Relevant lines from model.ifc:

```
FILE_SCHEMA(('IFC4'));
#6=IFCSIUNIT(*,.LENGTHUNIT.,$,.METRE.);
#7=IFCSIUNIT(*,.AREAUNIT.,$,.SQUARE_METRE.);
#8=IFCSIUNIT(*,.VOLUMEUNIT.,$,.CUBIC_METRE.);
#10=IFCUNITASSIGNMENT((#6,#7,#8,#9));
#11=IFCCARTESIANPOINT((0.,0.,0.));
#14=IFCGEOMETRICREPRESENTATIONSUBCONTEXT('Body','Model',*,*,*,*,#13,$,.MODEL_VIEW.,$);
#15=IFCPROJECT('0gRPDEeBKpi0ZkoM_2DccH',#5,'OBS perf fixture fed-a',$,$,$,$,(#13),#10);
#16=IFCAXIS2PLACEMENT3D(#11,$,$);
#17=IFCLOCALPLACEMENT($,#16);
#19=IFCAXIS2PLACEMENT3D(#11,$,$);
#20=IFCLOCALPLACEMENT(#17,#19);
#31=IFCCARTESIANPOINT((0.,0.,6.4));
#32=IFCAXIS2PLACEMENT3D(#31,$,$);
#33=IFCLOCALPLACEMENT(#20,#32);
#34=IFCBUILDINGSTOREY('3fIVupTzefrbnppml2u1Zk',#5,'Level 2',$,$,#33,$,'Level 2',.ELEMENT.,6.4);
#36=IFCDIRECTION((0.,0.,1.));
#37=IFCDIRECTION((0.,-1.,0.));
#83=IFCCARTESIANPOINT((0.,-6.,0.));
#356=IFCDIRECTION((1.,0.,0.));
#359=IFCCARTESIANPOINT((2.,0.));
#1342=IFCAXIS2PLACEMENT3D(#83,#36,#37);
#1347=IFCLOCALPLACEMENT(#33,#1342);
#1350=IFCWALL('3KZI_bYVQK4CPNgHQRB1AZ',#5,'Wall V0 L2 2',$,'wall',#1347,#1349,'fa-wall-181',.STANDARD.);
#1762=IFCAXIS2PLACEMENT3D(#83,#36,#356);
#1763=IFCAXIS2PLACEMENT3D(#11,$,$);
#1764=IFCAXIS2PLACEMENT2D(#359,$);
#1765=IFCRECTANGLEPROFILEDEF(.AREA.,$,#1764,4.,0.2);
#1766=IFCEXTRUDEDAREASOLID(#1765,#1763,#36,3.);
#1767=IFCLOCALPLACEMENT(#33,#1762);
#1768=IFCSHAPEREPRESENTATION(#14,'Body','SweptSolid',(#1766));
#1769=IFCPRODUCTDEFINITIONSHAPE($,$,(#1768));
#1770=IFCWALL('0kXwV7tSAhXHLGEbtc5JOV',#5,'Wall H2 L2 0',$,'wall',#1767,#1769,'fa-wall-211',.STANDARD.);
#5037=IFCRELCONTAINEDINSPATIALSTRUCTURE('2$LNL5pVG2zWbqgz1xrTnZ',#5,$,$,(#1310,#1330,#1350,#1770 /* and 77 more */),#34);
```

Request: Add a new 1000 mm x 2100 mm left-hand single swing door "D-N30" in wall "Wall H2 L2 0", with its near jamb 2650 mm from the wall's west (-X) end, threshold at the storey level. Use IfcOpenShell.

```python
import numpy as np
import ifcopenshell
import ifcopenshell.api.feature
import ifcopenshell.api.geometry
import ifcopenshell.api.root
import ifcopenshell.api.spatial
import ifcopenshell.geom
import ifcopenshell.util.element
import ifcopenshell.util.placement
import ifcopenshell.util.representation
import ifcopenshell.util.shape
import ifcopenshell.util.unit

model = ifcopenshell.open("model.ifc")
unit_scale = ifcopenshell.util.unit.calculate_unit_scale(model)
settings = ifcopenshell.geom.settings()


def volume(element):
    """Net volume in cubic metres, openings subtracted."""
    shape = ifcopenshell.geom.create_shape(settings, element)
    return ifcopenshell.util.shape.get_volume(shape.geometry)


wall = model.by_guid("0kXwV7tSAhXHLGEbtc5JOV")
storey = ifcopenshell.util.element.get_container(wall, ifc_class="IfcBuildingStorey")
context = ifcopenshell.util.representation.get_context(model, "Model", "Body", "MODEL_VIEW")
before = volume(wall)

width, height, from_end, sill = 1, 2.1, 2.65, 0.0  # metres

# The wall runs along its own X axis, and the end named is its -X end.
wall_shape = ifcopenshell.geom.create_shape(settings, wall)
x, y, z = ifcopenshell.util.shape.get_vertices(wall_shape.geometry).T
start = x.min() + from_end
face, thickness = float(y.min()), float(y.max() - y.min())
wall_matrix = ifcopenshell.util.placement.get_local_placement(wall.ObjectPlacement)
level = ifcopenshell.util.placement.get_local_placement(storey.ObjectPlacement)[2, 3]


def in_wall(x, y):
    """Placement at x, y metres in the wall's axes, at sill height."""
    matrix = wall_matrix.copy()
    matrix[:, 3] = wall_matrix @ np.array([x / unit_scale, y / unit_scale, 0.0, 1.0])
    matrix[2, 3] = level + sill / unit_scale
    return matrix


# Opening: a box that overshoots both wall faces by 50 mm.
opening = ifcopenshell.api.root.create_entity(model, ifc_class="IfcOpeningElement", predefined_type="OPENING")
box = ifcopenshell.api.geometry.add_wall_representation(
    model, context=context, length=width, height=height, thickness=thickness + 0.1
)
ifcopenshell.api.geometry.assign_representation(model, product=opening, representation=box)
ifcopenshell.api.geometry.edit_object_placement(model, product=opening, matrix=in_wall(start, face - 0.05), is_si=False)
ifcopenshell.api.feature.add_feature(model, feature=opening, element=wall)

door = ifcopenshell.api.root.create_entity(model, ifc_class="IfcDoor", name="D-N30", predefined_type="DOOR")
door.OverallWidth, door.OverallHeight = width / unit_scale, height / unit_scale
door.OperationType = "SINGLE_SWING_LEFT"
body = ifcopenshell.api.geometry.add_door_representation(
    model,
    context=context,
    overall_width=door.OverallWidth,
    overall_height=door.OverallHeight,
    operation_type="SINGLE_SWING_LEFT",
    lining_properties={"LiningDepth": thickness / unit_scale, "ThresholdDepth": thickness / unit_scale},
)
ifcopenshell.api.geometry.assign_representation(model, product=door, representation=body)
ifcopenshell.api.spatial.assign_container(model, products=[door], relating_structure=storey)
ifcopenshell.api.feature.add_filling(model, opening=opening, element=door)

# The lining spans the wall, so the door starts at the wall face.
ifcopenshell.api.geometry.edit_object_placement(model, product=door, matrix=in_wall(start, face), is_si=False)

after = volume(wall)

print(f"wall volume {before:.3f} -> {after:.3f} m3")

model.write("model_rev.ifc")
```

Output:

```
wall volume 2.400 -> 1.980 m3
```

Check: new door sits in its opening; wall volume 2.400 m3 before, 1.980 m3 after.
